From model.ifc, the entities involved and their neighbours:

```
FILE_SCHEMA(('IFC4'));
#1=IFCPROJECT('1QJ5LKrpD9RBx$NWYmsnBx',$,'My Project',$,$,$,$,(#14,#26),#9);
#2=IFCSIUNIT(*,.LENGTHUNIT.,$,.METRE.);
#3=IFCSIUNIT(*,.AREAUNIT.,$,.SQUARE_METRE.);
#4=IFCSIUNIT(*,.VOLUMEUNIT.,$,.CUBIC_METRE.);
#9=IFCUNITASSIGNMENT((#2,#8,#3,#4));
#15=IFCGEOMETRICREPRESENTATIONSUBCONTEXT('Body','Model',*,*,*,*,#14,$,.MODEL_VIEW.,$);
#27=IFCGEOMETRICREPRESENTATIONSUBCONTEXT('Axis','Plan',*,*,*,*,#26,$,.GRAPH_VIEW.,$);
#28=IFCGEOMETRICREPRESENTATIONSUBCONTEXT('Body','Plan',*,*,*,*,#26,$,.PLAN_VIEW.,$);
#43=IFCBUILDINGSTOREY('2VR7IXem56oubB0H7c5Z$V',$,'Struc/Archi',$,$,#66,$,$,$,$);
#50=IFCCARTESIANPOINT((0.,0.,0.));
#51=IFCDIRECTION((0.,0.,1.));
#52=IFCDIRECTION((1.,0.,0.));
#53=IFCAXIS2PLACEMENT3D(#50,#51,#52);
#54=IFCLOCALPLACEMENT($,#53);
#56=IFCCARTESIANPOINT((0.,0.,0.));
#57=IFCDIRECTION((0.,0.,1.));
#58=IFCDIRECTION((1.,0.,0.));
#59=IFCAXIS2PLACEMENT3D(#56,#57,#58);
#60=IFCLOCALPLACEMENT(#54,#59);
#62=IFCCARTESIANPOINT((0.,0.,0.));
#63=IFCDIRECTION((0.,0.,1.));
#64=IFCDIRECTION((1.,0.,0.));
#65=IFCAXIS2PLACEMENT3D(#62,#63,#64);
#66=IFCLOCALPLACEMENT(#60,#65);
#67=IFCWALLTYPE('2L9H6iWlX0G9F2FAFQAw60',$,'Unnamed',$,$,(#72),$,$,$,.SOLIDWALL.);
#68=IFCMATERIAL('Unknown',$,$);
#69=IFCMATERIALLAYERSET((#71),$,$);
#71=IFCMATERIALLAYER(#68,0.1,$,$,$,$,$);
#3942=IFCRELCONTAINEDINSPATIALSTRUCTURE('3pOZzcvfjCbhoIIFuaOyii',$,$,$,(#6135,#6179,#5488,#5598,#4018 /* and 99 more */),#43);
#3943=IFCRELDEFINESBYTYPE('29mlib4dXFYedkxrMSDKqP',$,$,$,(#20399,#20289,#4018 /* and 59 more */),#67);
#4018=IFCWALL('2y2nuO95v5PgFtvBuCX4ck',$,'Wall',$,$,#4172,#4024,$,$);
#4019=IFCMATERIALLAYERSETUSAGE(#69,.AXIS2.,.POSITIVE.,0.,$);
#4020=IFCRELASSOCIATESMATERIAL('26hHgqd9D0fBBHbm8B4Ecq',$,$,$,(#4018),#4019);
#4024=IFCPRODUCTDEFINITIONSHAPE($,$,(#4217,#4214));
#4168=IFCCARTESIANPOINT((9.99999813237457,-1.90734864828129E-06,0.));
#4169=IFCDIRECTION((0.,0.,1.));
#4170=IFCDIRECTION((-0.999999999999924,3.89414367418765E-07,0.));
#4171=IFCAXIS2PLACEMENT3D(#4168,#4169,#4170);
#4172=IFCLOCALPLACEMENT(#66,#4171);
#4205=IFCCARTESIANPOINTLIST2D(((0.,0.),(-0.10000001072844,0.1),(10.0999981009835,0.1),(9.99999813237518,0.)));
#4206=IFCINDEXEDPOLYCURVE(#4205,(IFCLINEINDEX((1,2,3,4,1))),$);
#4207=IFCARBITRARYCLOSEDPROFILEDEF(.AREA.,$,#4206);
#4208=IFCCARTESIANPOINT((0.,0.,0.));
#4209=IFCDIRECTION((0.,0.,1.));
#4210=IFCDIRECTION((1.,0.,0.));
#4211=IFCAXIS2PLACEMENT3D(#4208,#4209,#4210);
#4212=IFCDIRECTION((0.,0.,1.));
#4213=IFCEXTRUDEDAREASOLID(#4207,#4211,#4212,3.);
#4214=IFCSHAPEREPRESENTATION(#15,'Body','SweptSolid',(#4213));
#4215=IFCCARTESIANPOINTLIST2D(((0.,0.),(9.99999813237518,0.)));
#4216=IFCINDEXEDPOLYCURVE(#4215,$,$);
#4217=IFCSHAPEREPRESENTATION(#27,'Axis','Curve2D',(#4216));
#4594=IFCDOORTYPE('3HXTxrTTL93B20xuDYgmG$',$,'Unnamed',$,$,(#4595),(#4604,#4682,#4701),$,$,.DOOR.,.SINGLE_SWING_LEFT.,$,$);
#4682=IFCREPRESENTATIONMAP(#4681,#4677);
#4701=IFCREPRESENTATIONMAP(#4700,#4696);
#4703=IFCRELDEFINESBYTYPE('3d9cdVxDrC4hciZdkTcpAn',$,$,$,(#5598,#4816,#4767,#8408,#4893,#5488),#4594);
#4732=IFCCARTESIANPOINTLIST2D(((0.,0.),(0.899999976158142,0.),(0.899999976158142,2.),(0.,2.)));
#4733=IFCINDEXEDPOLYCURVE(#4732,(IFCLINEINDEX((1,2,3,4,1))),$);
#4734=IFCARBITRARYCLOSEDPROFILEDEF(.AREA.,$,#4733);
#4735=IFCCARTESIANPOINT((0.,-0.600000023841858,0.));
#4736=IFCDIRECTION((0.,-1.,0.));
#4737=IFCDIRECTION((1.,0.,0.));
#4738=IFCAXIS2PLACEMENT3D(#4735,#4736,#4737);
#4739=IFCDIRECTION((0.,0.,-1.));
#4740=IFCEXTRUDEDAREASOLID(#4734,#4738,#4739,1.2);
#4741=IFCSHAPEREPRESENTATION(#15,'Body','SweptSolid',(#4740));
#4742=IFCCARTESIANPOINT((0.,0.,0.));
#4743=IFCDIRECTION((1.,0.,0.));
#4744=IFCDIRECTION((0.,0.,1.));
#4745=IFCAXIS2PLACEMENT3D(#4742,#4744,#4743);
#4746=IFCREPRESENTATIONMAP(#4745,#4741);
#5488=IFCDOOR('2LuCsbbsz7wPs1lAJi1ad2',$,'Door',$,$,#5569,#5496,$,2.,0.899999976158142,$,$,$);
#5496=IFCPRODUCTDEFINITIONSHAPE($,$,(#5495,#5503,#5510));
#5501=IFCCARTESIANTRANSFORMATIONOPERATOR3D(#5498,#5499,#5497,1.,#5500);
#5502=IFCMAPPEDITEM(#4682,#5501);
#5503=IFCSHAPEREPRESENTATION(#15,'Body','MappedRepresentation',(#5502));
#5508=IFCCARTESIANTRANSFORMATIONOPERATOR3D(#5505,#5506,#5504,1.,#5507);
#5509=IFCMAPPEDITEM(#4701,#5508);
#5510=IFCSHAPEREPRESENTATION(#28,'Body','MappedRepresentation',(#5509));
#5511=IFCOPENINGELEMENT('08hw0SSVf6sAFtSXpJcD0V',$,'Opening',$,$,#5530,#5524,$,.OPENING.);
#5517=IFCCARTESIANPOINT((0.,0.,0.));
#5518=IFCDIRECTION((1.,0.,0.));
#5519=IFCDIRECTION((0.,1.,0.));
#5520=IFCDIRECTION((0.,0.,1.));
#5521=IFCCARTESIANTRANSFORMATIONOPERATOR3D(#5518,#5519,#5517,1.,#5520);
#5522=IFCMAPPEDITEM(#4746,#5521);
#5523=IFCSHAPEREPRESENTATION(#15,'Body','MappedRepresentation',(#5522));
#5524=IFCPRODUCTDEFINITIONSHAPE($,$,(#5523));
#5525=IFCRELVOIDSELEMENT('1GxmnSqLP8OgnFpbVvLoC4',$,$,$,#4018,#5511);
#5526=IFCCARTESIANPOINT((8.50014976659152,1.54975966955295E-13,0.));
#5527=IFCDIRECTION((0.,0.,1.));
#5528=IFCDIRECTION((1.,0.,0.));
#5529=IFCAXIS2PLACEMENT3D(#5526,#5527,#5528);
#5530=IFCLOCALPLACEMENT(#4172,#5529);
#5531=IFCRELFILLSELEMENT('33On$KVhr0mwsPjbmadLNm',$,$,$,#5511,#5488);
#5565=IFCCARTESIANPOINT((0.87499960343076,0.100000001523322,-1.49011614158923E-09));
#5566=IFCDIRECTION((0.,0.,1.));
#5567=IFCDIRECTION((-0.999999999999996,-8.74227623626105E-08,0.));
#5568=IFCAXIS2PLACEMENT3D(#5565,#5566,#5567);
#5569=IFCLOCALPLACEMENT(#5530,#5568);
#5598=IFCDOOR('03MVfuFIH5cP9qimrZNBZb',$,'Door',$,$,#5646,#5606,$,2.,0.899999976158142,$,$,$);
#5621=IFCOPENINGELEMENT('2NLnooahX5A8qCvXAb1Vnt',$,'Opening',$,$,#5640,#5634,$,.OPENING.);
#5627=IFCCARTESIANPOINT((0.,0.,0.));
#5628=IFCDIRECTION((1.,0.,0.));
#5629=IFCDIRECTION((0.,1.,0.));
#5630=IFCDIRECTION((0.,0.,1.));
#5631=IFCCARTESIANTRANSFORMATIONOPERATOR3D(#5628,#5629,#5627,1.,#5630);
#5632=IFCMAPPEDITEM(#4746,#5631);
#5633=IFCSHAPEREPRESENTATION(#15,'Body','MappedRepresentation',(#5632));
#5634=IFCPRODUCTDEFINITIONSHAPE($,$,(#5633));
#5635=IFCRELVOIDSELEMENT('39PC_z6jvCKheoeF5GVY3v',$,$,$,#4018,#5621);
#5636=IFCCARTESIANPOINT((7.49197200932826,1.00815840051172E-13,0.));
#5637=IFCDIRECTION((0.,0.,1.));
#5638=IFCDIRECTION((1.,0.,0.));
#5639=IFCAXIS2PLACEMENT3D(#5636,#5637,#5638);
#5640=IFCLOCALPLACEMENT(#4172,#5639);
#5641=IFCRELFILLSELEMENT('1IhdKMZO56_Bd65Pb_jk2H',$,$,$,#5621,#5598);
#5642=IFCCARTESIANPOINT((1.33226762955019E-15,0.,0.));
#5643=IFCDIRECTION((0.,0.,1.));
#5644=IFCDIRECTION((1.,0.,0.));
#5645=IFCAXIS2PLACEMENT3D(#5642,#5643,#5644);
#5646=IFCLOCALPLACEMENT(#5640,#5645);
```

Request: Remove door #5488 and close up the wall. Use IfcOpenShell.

```python
import ifcopenshell
import ifcopenshell.api.feature
import ifcopenshell.api.root
import ifcopenshell.geom
import ifcopenshell.util.shape

model = ifcopenshell.open("model.ifc")
settings = ifcopenshell.geom.settings()


def volume(element):
    """Net volume in cubic metres, openings subtracted."""
    shape = ifcopenshell.geom.create_shape(settings, element)
    return ifcopenshell.util.shape.get_volume(shape.geometry)


door = model.by_guid("2LuCsbbsz7wPs1lAJi1ad2")
opening = door.FillsVoids[0].RelatingOpeningElement
wall = opening.VoidsElements[0].RelatingBuildingElement
before = volume(wall)

ifcopenshell.api.root.remove_product(model, product=door)
ifcopenshell.api.feature.remove_feature(model, feature=opening)

after = volume(wall)

print(f"wall volume {before:.3f} -> {after:.3f} m3")

model.write("model_updated.ifc")
```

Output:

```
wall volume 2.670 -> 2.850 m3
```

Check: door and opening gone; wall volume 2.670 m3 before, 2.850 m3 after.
